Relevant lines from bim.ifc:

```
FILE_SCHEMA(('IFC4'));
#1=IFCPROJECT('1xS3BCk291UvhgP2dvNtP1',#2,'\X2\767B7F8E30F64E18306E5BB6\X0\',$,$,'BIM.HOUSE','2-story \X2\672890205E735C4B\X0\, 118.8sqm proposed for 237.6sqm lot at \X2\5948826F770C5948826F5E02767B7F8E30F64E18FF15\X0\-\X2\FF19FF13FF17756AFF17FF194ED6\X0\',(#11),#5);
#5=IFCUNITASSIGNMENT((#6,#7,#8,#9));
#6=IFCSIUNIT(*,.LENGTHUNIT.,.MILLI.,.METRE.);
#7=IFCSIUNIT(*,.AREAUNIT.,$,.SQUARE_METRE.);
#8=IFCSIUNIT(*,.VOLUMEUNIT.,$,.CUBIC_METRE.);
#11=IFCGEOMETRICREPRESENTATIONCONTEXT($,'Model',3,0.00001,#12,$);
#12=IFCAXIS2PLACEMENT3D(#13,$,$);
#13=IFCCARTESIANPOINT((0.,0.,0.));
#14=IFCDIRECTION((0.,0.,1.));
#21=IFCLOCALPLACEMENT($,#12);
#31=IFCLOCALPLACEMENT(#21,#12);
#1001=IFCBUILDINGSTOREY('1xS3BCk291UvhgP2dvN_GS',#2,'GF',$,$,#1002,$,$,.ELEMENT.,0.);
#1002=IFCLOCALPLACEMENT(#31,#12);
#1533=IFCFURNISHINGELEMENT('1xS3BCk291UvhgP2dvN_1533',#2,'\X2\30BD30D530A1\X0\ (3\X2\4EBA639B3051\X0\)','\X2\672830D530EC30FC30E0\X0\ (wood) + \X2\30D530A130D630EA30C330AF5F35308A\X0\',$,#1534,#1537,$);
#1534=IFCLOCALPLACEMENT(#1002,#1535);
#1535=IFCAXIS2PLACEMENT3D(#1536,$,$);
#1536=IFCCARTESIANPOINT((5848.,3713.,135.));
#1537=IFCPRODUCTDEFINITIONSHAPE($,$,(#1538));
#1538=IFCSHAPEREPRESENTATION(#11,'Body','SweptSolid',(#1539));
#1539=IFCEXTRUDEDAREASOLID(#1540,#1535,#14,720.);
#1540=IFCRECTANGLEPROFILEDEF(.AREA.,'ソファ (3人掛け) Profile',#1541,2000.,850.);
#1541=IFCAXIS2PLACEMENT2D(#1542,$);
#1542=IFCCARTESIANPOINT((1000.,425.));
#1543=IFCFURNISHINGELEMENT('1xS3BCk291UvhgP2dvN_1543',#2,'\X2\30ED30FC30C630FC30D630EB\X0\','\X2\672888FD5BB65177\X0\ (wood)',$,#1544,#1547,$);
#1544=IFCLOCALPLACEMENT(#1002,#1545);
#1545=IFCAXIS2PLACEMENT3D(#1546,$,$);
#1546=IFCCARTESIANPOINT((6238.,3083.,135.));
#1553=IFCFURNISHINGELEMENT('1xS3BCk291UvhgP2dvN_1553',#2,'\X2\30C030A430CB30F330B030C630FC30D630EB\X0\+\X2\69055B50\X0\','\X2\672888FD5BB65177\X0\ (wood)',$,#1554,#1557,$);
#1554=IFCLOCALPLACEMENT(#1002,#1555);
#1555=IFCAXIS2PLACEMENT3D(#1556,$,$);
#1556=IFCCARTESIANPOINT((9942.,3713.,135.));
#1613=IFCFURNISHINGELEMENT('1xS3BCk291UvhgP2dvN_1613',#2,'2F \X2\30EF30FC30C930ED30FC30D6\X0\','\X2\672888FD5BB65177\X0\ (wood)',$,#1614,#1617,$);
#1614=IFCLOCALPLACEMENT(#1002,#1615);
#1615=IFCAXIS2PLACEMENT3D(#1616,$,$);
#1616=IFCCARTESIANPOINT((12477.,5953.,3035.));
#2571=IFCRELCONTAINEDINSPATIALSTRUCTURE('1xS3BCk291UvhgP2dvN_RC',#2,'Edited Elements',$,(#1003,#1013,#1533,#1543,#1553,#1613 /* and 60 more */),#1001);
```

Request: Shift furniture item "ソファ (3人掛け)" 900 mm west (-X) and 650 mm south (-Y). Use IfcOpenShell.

```python
import ifcopenshell
import ifcopenshell.api.geometry
import ifcopenshell.util.placement
import ifcopenshell.util.unit

model = ifcopenshell.open("bim.ifc")
unit_scale = ifcopenshell.util.unit.calculate_unit_scale(model)

item = model.by_id(1533)
matrix = ifcopenshell.util.placement.get_local_placement(item.ObjectPlacement)
matrix[0, 3] -= 0.9 / unit_scale
matrix[1, 3] -= 0.65 / unit_scale
ifcopenshell.api.geometry.edit_object_placement(model, product=item, matrix=matrix, is_si=False)

print(ifcopenshell.util.placement.get_local_placement(item.ObjectPlacement).round(3) + 0.0)

model.write("bim_edited.ifc")
```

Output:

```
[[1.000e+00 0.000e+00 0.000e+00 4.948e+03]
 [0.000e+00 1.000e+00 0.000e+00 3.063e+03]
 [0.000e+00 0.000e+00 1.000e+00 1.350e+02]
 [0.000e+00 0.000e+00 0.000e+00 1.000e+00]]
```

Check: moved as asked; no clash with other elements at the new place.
